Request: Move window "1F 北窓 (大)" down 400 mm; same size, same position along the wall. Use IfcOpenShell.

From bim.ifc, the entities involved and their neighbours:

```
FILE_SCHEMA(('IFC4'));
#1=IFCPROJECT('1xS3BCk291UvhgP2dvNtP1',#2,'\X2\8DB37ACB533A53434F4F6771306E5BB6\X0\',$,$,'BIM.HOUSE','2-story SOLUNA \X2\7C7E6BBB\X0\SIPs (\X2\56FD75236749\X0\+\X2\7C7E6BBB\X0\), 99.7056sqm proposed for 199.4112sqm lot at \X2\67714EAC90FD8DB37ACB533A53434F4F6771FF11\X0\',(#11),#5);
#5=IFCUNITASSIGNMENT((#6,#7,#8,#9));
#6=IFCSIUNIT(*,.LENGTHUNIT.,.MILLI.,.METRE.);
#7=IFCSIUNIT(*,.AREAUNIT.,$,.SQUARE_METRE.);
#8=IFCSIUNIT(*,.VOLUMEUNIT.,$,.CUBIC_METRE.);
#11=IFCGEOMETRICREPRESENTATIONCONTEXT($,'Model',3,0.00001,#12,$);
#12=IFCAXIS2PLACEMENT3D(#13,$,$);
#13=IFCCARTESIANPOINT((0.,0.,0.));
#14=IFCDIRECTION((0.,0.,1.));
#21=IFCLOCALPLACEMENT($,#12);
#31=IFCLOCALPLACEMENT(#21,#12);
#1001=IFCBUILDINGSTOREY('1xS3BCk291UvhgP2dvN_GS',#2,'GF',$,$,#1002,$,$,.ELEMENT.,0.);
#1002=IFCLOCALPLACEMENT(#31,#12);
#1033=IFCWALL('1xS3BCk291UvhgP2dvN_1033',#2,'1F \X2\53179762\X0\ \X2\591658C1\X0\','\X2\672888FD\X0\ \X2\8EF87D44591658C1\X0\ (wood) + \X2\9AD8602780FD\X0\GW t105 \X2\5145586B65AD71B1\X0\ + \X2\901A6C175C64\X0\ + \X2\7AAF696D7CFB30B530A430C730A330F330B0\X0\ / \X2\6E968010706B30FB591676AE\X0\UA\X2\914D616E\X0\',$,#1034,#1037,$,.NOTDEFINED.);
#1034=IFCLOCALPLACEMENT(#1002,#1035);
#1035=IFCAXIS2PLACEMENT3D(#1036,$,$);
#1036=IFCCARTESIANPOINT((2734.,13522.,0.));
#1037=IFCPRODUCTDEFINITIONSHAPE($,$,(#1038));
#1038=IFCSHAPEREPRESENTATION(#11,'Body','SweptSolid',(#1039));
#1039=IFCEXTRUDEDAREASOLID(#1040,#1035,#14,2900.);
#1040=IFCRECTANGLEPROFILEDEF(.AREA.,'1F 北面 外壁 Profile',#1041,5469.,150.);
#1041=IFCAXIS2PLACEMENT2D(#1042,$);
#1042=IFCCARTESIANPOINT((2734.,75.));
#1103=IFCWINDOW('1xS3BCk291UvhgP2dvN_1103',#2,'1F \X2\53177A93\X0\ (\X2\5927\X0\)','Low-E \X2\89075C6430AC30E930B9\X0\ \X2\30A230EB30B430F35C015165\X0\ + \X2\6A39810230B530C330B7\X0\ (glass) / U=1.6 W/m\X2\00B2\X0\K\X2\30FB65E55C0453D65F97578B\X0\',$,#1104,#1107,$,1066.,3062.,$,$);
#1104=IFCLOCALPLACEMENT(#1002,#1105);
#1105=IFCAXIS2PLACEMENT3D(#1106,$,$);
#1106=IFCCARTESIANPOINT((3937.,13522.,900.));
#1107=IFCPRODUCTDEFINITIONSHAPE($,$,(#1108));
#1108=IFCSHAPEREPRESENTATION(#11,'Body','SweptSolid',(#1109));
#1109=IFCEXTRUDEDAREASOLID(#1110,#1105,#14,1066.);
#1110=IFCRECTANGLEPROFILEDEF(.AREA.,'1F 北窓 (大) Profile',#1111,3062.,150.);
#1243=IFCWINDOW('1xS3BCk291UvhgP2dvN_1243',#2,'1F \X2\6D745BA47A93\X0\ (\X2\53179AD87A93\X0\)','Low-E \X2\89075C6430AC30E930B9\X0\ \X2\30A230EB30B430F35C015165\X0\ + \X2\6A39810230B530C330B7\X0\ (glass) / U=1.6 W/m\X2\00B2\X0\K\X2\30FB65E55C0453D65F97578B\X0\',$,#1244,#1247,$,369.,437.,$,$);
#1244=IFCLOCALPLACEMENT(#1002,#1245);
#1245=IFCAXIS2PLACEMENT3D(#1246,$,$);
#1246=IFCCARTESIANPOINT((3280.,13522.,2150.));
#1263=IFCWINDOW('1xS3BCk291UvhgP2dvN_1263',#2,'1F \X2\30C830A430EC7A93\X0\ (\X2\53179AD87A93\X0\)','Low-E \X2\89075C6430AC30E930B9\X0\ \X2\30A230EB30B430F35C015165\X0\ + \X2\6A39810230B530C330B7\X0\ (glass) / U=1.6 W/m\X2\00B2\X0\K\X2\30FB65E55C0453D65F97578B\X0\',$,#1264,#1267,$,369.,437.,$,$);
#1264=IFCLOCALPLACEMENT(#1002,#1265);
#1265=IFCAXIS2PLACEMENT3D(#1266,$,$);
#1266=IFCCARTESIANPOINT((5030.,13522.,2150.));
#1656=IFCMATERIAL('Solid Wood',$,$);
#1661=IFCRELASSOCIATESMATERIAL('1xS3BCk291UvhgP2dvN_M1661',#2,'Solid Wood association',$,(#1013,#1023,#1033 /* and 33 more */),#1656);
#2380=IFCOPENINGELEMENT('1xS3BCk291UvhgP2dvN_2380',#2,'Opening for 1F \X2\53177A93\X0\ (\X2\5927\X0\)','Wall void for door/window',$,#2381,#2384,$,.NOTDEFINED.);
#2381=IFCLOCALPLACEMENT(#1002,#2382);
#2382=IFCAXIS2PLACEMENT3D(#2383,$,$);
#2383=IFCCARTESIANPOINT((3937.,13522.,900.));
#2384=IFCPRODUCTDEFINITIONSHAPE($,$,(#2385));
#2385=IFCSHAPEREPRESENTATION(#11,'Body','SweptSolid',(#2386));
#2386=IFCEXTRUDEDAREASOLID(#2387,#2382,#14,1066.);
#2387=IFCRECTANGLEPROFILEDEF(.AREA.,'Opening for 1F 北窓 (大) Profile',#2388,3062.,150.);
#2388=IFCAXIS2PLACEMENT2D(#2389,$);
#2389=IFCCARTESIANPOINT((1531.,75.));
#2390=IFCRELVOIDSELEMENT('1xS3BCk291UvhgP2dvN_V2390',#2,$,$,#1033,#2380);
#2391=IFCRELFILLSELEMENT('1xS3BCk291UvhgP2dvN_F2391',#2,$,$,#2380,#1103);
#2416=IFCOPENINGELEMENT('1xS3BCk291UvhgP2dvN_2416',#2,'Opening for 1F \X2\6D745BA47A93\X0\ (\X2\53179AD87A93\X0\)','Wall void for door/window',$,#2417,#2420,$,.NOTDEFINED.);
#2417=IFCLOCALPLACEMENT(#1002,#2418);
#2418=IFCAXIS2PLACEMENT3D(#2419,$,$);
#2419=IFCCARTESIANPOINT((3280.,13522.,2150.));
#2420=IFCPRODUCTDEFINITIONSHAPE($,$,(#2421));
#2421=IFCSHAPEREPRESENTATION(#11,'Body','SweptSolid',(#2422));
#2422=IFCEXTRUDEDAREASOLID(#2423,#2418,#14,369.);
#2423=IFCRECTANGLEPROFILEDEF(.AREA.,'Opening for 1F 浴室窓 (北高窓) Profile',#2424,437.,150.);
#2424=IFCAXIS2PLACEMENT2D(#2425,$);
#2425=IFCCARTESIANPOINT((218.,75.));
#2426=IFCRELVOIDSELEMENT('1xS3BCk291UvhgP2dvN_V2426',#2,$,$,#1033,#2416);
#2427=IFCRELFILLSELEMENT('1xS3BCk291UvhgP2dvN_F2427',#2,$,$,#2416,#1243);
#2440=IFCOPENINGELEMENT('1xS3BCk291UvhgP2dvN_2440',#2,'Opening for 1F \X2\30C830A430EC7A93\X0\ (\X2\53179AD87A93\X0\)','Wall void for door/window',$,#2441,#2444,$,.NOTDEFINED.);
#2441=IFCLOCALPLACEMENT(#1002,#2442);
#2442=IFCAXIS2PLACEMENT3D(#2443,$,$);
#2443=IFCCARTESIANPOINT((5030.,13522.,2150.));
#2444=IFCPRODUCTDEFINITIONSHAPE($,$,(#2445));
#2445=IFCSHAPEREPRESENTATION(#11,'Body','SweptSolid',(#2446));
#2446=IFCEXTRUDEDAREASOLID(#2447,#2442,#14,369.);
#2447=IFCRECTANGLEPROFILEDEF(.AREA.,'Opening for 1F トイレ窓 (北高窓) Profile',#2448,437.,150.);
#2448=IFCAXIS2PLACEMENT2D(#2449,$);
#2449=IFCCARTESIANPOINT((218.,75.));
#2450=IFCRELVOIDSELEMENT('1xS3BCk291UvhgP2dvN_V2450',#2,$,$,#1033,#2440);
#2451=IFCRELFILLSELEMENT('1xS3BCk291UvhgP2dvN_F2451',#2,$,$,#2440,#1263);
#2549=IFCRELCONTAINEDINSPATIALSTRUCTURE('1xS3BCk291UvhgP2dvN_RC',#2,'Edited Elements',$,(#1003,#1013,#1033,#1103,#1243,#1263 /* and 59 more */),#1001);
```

```python
import numpy as np
import ifcopenshell
import ifcopenshell.api.geometry
import ifcopenshell.util.placement
import ifcopenshell.util.unit

model = ifcopenshell.open("bim.ifc")
unit_scale = ifcopenshell.util.unit.calculate_unit_scale(model)

window = model.by_id(1103)
opening = window.FillsVoids[0].RelatingOpeningElement
dz = -400.0

shift = np.array([0.0, 0.0, dz])
# The window is not placed relative to its opening, so move both.
for product in (opening, window):
    matrix = ifcopenshell.util.placement.get_local_placement(product.ObjectPlacement)
    matrix[:3, 3] += shift
    ifcopenshell.api.geometry.edit_object_placement(model, product=product, matrix=matrix, is_si=False)

print(f"moved by {dz * unit_scale:+.3f} m")

model.write("bim_v2.ifc")
```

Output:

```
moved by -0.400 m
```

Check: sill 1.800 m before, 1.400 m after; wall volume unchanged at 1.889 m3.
